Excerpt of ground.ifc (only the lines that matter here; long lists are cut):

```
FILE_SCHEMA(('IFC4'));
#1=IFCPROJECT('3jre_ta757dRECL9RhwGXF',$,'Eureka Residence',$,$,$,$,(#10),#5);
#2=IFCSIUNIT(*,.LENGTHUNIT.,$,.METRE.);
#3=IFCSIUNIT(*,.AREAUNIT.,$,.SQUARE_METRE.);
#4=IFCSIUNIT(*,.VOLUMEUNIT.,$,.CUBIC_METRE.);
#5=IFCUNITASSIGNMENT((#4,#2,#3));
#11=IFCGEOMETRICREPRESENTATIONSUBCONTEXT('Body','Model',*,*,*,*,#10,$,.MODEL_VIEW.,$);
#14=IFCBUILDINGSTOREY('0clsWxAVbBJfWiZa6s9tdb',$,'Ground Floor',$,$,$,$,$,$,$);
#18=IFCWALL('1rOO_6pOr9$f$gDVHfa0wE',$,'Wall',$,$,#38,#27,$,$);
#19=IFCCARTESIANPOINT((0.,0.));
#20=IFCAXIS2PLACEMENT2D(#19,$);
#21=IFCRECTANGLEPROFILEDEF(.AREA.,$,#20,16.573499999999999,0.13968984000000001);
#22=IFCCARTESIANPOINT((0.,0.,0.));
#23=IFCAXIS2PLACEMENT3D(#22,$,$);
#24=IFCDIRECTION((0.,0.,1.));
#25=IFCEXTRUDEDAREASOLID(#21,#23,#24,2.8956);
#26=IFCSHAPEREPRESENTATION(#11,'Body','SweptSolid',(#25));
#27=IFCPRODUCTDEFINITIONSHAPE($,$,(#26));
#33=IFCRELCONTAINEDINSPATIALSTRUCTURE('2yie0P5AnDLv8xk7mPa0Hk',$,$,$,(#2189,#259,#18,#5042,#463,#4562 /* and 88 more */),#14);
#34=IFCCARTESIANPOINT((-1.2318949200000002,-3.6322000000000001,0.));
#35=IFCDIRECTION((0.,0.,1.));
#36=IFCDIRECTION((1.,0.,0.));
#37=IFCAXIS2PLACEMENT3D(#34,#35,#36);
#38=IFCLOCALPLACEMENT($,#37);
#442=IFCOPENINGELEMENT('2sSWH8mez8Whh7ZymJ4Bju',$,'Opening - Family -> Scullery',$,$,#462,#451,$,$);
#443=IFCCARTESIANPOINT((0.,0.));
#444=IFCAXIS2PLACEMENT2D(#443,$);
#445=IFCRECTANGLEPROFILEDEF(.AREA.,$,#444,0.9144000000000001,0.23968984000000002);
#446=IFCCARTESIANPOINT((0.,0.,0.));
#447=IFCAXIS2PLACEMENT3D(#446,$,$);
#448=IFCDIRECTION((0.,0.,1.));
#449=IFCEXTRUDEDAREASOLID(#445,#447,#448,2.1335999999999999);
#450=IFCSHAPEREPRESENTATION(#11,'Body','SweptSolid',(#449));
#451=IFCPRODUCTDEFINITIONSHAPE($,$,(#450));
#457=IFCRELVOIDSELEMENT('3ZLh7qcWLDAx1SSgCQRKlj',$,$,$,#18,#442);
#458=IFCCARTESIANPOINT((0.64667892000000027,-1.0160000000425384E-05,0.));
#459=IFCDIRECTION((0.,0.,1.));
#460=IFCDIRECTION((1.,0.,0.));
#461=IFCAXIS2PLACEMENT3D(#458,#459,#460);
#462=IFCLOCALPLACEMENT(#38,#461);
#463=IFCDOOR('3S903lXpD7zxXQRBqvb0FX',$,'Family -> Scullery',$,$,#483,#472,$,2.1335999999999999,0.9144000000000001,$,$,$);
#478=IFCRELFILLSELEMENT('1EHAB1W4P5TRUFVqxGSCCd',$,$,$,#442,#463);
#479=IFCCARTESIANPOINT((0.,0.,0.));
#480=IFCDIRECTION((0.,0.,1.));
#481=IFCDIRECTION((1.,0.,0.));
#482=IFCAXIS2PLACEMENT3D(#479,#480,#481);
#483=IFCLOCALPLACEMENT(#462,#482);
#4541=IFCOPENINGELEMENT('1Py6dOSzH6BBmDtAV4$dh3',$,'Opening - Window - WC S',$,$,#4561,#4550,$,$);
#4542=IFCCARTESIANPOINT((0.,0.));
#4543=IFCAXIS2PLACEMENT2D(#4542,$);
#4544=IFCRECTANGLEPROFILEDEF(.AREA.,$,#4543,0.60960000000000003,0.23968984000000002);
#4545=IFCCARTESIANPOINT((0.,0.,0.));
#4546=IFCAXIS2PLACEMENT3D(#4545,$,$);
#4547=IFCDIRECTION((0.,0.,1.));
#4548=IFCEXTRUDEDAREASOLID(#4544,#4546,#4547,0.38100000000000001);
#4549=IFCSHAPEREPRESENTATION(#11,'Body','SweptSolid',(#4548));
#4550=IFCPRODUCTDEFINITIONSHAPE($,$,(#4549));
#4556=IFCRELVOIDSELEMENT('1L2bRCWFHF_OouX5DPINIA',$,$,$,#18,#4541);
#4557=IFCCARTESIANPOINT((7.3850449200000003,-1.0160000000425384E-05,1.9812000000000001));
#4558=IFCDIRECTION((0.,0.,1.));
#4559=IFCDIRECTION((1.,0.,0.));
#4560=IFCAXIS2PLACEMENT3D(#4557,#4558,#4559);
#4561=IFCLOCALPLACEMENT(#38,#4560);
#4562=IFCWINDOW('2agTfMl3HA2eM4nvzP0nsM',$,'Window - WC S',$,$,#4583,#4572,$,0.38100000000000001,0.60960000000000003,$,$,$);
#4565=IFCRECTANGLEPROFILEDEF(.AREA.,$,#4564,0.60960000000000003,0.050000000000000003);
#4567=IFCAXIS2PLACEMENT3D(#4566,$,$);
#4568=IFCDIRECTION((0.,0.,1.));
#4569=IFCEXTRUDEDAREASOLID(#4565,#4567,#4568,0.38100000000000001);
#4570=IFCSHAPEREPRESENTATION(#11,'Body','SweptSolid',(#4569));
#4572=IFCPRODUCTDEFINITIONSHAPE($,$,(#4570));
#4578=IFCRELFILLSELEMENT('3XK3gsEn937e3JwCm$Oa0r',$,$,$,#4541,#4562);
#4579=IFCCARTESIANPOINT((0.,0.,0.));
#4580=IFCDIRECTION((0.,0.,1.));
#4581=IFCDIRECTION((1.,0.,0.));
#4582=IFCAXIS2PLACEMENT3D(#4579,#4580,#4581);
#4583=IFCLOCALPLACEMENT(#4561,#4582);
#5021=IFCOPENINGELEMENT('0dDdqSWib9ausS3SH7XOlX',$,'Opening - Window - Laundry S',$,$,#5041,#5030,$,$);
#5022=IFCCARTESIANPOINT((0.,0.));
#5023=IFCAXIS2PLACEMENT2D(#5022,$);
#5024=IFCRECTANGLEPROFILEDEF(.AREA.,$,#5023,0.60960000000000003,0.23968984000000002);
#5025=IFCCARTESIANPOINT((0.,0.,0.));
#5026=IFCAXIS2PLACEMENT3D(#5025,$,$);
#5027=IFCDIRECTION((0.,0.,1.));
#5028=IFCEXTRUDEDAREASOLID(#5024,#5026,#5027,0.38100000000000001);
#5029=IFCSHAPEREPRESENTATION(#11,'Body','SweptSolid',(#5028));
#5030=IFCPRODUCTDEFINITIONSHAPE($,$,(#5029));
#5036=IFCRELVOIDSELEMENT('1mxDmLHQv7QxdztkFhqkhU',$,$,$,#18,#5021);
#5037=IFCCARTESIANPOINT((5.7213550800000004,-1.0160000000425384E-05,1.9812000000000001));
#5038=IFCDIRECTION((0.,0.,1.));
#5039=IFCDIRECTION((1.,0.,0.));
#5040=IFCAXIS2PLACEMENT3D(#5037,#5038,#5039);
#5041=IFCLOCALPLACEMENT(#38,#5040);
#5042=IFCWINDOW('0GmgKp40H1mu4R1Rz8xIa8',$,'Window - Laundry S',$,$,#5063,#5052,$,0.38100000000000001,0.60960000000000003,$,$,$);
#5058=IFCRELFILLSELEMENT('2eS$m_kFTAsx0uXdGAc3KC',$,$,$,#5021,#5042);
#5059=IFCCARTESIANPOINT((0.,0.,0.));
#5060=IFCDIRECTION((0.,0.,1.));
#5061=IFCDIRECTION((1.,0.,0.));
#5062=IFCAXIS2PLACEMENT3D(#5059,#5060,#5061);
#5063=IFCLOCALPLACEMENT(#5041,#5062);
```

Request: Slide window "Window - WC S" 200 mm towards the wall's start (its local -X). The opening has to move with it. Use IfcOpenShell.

```python
import ifcopenshell
import ifcopenshell.api.geometry
import ifcopenshell.util.placement
import ifcopenshell.util.unit

model = ifcopenshell.open("ground.ifc")
unit_scale = ifcopenshell.util.unit.calculate_unit_scale(model)

window = model.by_id(4562)
opening = window.FillsVoids[0].RelatingOpeningElement
wall = opening.VoidsElements[0].RelatingBuildingElement

wall_matrix = ifcopenshell.util.placement.get_local_placement(wall.ObjectPlacement)
shift = wall_matrix[:3, 0] * -0.2 / unit_scale
before = ifcopenshell.util.placement.get_local_placement(window.ObjectPlacement)[:3, 3].copy()

# The window is placed relative to its opening, so it follows when the opening moves.
matrix = ifcopenshell.util.placement.get_local_placement(opening.ObjectPlacement)
matrix[:3, 3] += shift
ifcopenshell.api.geometry.edit_object_placement(
    model, product=opening, matrix=matrix, is_si=False, should_transform_children=True
)

after = ifcopenshell.util.placement.get_local_placement(window.ObjectPlacement)[:3, 3]
print("window moved by", (after - before).round(3) + 0.0)

model.write("ground-out.ifc")
```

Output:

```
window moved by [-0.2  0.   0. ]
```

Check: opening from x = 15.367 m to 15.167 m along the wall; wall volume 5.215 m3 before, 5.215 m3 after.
